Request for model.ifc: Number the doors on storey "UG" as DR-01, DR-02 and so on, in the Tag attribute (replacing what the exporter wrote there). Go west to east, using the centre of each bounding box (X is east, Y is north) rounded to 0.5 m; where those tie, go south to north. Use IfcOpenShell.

First a look at what the model holds.

```python
import ifcopenshell
import ifcopenshell.util.element
import ifcopenshell.util.placement

model = ifcopenshell.open("model.ifc")
print(model.schema)
storey = next(s for s in model.by_type("IfcBuildingStorey") if s.Name == "UG")
doors = [e for e in ifcopenshell.util.element.get_decomposition(storey) if e.is_a("IfcDoor")]
for e in sorted(doors, key=lambda e: e.id()):
    origin = ifcopenshell.util.placement.get_local_placement(e.ObjectPlacement)[:3, 3]
    print(e.id(), e.Tag, e.Name, origin.round(2) + 0.0, sep=" | ")
```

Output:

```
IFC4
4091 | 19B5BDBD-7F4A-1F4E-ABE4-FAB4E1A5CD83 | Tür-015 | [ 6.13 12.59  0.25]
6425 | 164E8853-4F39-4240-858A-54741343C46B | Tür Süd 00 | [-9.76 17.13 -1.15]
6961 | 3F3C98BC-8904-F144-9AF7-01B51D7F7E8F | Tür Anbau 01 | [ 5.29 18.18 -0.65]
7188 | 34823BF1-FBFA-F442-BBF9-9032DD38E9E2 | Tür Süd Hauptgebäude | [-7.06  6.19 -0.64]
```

```python
import ifcopenshell
import ifcopenshell.geom
import ifcopenshell.util.element
import ifcopenshell.util.shape

model = ifcopenshell.open("model.ifc")
settings = ifcopenshell.geom.settings()
settings.set("use-world-coords", True)


def centre(element):
    shape = ifcopenshell.geom.create_shape(settings, element)
    return ifcopenshell.util.shape.get_bbox_centroid(shape.geometry)


storey = next(s for s in model.by_type("IfcBuildingStorey") if s.Name == "UG")
doors = [e for e in ifcopenshell.util.element.get_decomposition(storey) if e.is_a("IfcDoor")]

# Insertion points can sit at a corner or the storey origin, so sort by the geometry (in metres).
centres = {e: centre(e) for e in doors}
doors.sort(key=lambda e: (round(centres[e][0] / 0.5), centres[e][1]))

for i, e in enumerate(doors, start=1):
    number = f"DR-{i:02d}"
    e.Tag = number
    print(e.id(), number)

model.write("model-out.ifc")
```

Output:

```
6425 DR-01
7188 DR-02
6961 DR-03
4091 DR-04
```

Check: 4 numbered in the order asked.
